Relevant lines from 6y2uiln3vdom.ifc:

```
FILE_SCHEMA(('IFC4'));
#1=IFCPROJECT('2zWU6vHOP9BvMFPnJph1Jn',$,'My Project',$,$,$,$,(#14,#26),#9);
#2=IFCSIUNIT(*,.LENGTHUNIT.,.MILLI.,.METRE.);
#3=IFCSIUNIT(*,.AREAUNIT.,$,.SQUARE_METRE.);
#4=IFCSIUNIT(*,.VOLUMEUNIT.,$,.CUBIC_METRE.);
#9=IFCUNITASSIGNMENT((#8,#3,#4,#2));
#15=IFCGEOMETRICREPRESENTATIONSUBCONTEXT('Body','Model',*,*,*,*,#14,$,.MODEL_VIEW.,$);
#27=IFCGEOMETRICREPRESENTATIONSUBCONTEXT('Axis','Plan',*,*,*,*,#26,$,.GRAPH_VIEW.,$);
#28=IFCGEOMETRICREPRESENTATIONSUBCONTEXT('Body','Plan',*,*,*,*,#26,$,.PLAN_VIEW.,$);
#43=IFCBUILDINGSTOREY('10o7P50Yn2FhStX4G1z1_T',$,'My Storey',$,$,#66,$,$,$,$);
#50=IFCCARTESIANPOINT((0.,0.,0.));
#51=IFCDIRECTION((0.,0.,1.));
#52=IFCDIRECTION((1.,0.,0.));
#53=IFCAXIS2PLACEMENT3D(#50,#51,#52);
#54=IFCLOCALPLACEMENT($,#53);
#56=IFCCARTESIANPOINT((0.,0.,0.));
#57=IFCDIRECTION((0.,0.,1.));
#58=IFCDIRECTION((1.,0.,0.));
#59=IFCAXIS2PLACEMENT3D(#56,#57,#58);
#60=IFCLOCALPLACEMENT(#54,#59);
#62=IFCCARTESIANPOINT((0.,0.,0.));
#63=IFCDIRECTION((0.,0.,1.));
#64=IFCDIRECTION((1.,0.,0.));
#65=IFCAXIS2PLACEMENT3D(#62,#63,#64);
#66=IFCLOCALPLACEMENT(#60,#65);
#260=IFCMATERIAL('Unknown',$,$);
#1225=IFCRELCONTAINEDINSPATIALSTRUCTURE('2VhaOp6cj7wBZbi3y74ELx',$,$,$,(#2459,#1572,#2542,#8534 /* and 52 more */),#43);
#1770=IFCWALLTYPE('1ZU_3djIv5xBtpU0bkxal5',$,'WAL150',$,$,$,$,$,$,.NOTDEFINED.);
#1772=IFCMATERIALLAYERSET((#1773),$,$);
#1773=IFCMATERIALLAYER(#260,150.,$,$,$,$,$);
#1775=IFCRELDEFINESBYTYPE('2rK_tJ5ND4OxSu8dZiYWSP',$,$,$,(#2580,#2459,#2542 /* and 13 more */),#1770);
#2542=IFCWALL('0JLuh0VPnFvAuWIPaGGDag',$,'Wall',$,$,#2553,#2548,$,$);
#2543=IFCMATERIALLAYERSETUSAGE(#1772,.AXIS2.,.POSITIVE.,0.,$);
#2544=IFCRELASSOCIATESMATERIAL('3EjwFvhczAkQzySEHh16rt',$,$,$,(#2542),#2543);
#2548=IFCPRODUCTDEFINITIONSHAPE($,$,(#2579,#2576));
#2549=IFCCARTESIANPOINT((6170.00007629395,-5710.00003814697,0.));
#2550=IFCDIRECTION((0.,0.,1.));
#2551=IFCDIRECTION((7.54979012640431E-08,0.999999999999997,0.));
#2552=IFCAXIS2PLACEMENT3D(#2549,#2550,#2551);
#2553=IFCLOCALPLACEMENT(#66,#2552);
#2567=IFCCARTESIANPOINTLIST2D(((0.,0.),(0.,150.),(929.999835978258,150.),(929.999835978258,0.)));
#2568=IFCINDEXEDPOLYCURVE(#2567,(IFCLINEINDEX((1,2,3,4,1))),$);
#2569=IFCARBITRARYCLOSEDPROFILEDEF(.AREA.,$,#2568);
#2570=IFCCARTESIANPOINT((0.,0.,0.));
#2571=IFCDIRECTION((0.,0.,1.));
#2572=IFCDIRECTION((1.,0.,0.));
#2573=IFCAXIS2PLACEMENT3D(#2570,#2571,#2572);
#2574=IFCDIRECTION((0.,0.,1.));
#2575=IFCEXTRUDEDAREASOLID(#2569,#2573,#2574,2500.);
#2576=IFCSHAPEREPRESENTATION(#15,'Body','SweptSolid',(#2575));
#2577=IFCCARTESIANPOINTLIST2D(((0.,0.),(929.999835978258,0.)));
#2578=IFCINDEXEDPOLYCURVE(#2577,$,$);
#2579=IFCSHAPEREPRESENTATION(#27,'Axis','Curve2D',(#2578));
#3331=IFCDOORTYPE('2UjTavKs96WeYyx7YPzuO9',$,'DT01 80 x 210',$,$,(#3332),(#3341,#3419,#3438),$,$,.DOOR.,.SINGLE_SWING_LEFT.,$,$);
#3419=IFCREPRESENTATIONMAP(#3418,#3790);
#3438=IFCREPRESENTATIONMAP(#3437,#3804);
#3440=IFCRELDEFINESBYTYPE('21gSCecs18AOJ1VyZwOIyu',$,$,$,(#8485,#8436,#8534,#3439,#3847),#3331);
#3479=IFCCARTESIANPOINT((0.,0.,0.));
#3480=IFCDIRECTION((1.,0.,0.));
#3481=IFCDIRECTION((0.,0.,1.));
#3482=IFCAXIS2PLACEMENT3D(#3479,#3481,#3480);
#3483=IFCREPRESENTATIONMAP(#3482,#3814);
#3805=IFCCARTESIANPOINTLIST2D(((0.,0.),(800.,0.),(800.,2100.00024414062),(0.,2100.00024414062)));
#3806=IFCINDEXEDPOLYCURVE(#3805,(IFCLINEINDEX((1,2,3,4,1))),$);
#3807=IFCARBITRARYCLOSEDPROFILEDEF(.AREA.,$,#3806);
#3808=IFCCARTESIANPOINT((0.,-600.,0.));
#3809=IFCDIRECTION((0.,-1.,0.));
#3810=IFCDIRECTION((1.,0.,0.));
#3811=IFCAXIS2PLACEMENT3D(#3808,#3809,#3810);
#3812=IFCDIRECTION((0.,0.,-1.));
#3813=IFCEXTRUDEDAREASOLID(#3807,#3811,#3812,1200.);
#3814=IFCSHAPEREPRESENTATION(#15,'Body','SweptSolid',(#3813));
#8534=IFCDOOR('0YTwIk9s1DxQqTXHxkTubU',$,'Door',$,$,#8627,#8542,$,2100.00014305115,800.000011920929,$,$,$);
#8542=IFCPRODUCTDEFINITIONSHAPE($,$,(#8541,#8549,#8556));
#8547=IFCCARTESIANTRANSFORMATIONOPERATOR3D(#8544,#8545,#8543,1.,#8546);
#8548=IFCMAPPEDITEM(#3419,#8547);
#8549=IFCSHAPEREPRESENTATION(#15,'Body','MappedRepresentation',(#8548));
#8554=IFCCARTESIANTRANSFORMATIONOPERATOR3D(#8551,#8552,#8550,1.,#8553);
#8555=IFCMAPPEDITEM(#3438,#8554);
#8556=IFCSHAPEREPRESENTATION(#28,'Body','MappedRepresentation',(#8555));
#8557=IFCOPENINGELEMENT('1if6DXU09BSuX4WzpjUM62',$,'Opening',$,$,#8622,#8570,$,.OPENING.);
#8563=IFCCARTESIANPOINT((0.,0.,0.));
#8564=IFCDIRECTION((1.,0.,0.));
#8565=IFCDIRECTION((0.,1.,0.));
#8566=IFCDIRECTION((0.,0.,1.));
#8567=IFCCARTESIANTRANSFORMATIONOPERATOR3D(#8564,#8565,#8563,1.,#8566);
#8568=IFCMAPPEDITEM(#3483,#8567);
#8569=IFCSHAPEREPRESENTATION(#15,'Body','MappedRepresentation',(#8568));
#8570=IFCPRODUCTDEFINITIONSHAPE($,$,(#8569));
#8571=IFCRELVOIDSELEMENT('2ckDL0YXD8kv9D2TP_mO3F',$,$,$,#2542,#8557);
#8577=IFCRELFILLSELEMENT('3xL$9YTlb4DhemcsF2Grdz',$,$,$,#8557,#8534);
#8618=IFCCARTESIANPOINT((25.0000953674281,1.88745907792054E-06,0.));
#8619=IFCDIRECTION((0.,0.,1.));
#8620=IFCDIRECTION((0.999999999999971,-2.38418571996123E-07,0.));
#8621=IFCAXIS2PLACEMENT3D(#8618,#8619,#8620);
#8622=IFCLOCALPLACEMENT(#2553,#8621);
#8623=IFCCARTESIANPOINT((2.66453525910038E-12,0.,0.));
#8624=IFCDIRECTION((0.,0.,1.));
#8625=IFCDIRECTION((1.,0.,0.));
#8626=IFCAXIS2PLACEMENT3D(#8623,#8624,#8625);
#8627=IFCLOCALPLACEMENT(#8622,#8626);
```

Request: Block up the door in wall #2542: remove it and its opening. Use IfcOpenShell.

```python
import ifcopenshell
import ifcopenshell.api.feature
import ifcopenshell.api.root
import ifcopenshell.geom
import ifcopenshell.util.shape

model = ifcopenshell.open("6y2uiln3vdom.ifc")
settings = ifcopenshell.geom.settings()


def volume(element):
    """Net volume in cubic metres, openings subtracted."""
    shape = ifcopenshell.geom.create_shape(settings, element)
    return ifcopenshell.util.shape.get_volume(shape.geometry)


door = model.by_guid("0YTwIk9s1DxQqTXHxkTubU")
opening = door.FillsVoids[0].RelatingOpeningElement
wall = opening.VoidsElements[0].RelatingBuildingElement
before = volume(wall)

ifcopenshell.api.root.remove_product(model, product=door)
ifcopenshell.api.feature.remove_feature(model, feature=opening)

after = volume(wall)

print(f"wall volume {before:.3f} -> {after:.3f} m3")

model.write("6y2uiln3vdom_updated.ifc")
```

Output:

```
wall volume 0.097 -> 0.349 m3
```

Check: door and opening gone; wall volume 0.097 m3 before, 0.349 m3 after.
